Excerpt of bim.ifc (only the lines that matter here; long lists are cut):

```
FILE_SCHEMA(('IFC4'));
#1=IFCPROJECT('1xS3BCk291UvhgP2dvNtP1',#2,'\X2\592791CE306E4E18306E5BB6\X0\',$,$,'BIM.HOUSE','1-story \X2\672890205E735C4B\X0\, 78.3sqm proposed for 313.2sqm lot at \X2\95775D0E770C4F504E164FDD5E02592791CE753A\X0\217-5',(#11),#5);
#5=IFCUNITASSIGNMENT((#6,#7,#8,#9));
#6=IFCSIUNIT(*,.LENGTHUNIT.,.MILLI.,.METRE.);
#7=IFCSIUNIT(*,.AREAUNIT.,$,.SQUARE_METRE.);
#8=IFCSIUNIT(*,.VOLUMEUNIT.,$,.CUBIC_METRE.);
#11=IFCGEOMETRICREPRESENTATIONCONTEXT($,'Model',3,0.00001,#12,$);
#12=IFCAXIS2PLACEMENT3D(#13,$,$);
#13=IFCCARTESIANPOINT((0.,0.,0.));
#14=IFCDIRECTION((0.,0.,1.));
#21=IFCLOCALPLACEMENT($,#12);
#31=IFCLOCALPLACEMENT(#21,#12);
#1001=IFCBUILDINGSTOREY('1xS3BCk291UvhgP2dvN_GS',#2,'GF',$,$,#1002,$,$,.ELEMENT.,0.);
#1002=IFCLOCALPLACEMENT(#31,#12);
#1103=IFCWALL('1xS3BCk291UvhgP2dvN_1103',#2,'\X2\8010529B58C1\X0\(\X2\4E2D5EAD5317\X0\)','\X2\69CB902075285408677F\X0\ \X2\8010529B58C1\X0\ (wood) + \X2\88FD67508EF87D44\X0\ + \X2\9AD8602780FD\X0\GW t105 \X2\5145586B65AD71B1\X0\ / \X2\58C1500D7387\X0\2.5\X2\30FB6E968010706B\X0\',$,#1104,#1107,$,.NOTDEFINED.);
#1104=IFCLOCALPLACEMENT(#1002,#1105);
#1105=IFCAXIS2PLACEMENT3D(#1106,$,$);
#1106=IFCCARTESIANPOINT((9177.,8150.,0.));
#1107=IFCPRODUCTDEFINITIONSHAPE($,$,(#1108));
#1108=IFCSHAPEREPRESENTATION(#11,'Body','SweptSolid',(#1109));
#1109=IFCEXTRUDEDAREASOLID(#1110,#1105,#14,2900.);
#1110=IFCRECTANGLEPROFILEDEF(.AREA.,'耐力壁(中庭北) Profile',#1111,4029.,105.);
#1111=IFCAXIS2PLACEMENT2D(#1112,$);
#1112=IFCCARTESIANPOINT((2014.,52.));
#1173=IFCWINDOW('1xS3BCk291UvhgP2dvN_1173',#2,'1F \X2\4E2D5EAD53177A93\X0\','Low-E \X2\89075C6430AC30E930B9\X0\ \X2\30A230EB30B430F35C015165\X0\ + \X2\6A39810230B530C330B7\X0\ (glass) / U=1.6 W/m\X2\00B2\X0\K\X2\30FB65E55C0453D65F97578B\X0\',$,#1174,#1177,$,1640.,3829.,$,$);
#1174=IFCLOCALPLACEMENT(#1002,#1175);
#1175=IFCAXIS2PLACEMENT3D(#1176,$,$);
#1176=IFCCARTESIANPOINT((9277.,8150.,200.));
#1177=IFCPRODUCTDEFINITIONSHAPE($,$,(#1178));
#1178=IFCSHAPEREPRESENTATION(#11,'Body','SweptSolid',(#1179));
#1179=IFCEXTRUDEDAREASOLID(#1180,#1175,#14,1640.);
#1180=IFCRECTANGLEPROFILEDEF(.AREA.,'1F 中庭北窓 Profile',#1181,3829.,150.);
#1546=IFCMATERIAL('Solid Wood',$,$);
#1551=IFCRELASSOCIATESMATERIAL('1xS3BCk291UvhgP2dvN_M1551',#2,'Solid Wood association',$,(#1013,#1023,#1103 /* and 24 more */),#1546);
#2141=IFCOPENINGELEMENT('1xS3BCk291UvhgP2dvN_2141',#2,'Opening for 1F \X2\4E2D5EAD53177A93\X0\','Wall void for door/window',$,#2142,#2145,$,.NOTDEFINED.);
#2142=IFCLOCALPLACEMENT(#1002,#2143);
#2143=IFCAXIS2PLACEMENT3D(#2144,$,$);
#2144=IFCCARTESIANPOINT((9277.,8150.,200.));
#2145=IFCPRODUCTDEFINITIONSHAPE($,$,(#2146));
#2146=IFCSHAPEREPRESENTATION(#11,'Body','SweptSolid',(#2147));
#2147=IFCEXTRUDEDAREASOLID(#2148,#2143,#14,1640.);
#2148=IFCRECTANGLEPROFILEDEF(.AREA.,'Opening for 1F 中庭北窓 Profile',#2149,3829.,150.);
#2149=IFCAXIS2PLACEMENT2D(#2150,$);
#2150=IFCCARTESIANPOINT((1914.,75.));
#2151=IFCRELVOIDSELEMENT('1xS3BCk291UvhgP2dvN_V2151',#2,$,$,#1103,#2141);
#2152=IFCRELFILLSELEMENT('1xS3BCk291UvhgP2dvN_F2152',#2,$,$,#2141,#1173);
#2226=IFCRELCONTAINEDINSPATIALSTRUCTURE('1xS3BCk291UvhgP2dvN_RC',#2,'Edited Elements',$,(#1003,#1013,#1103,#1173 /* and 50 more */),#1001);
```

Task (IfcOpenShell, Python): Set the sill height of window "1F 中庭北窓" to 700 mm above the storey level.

```python
import numpy as np
import ifcopenshell
import ifcopenshell.api.geometry
import ifcopenshell.geom
import ifcopenshell.util.element
import ifcopenshell.util.placement
import ifcopenshell.util.shape
import ifcopenshell.util.unit

model = ifcopenshell.open("bim.ifc")
unit_scale = ifcopenshell.util.unit.calculate_unit_scale(model)

window = model.by_guid("1xS3BCk291UvhgP2dvN_1173")
opening = window.FillsVoids[0].RelatingOpeningElement
storey = ifcopenshell.util.element.get_container(window, ifc_class="IfcBuildingStorey")
level = ifcopenshell.util.placement.get_local_placement(storey.ObjectPlacement)[2, 3]

# The opening's origin need not be at the sill, so measure its lowest point.
shape = ifcopenshell.geom.create_shape(ifcopenshell.geom.settings(), opening)
bottom = ifcopenshell.util.shape.get_shape_bottom_elevation(shape, shape.geometry) / unit_scale
dz = level + 0.7 / unit_scale - bottom

shift = np.array([0.0, 0.0, dz])
# The window is not placed relative to its opening, so move both.
for product in (opening, window):
    matrix = ifcopenshell.util.placement.get_local_placement(product.ObjectPlacement)
    matrix[:3, 3] += shift
    ifcopenshell.api.geometry.edit_object_placement(model, product=product, matrix=matrix, is_si=False)

print(f"moved by {dz * unit_scale:+.3f} m")

model.write("bim-out.ifc")
```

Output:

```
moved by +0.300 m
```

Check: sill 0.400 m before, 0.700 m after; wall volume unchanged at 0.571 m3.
